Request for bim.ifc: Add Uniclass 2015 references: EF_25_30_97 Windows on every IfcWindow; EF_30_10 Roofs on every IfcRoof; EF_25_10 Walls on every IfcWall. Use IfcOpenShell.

First a look at what the model holds.

```python
import ifcopenshell

model = ifcopenshell.open("bim.ifc")
print(model.schema)
print("classifications:", [c.Name for c in model.by_type("IfcClassification")])
for ifc_class in ("IfcDoor", "IfcRoof", "IfcStair", "IfcWall", "IfcWindow"):
    print(ifc_class, len(model.by_type(ifc_class)))
```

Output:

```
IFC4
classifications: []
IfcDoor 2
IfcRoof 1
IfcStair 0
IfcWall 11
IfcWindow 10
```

```python
import ifcopenshell
import ifcopenshell.api.classification

model = ifcopenshell.open("bim.ifc")

system = ifcopenshell.api.classification.add_classification(model, classification="Uniclass 2015")

codes = {
    "IfcWindow": ("EF_25_30_97", "Windows"),
    "IfcRoof": ("EF_30_10", "Roofs"),
    "IfcWall": ("EF_25_10", "Walls"),
}
for ifc_class, (code, name) in codes.items():
    products = model.by_type(ifc_class)
    ifcopenshell.api.classification.add_reference(
        model, products=products, classification=system, identification=code, name=name
    )
    print(code, len(products))

model.write("bim_rev.ifc")
```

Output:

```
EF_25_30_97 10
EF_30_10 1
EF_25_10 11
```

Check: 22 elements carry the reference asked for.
